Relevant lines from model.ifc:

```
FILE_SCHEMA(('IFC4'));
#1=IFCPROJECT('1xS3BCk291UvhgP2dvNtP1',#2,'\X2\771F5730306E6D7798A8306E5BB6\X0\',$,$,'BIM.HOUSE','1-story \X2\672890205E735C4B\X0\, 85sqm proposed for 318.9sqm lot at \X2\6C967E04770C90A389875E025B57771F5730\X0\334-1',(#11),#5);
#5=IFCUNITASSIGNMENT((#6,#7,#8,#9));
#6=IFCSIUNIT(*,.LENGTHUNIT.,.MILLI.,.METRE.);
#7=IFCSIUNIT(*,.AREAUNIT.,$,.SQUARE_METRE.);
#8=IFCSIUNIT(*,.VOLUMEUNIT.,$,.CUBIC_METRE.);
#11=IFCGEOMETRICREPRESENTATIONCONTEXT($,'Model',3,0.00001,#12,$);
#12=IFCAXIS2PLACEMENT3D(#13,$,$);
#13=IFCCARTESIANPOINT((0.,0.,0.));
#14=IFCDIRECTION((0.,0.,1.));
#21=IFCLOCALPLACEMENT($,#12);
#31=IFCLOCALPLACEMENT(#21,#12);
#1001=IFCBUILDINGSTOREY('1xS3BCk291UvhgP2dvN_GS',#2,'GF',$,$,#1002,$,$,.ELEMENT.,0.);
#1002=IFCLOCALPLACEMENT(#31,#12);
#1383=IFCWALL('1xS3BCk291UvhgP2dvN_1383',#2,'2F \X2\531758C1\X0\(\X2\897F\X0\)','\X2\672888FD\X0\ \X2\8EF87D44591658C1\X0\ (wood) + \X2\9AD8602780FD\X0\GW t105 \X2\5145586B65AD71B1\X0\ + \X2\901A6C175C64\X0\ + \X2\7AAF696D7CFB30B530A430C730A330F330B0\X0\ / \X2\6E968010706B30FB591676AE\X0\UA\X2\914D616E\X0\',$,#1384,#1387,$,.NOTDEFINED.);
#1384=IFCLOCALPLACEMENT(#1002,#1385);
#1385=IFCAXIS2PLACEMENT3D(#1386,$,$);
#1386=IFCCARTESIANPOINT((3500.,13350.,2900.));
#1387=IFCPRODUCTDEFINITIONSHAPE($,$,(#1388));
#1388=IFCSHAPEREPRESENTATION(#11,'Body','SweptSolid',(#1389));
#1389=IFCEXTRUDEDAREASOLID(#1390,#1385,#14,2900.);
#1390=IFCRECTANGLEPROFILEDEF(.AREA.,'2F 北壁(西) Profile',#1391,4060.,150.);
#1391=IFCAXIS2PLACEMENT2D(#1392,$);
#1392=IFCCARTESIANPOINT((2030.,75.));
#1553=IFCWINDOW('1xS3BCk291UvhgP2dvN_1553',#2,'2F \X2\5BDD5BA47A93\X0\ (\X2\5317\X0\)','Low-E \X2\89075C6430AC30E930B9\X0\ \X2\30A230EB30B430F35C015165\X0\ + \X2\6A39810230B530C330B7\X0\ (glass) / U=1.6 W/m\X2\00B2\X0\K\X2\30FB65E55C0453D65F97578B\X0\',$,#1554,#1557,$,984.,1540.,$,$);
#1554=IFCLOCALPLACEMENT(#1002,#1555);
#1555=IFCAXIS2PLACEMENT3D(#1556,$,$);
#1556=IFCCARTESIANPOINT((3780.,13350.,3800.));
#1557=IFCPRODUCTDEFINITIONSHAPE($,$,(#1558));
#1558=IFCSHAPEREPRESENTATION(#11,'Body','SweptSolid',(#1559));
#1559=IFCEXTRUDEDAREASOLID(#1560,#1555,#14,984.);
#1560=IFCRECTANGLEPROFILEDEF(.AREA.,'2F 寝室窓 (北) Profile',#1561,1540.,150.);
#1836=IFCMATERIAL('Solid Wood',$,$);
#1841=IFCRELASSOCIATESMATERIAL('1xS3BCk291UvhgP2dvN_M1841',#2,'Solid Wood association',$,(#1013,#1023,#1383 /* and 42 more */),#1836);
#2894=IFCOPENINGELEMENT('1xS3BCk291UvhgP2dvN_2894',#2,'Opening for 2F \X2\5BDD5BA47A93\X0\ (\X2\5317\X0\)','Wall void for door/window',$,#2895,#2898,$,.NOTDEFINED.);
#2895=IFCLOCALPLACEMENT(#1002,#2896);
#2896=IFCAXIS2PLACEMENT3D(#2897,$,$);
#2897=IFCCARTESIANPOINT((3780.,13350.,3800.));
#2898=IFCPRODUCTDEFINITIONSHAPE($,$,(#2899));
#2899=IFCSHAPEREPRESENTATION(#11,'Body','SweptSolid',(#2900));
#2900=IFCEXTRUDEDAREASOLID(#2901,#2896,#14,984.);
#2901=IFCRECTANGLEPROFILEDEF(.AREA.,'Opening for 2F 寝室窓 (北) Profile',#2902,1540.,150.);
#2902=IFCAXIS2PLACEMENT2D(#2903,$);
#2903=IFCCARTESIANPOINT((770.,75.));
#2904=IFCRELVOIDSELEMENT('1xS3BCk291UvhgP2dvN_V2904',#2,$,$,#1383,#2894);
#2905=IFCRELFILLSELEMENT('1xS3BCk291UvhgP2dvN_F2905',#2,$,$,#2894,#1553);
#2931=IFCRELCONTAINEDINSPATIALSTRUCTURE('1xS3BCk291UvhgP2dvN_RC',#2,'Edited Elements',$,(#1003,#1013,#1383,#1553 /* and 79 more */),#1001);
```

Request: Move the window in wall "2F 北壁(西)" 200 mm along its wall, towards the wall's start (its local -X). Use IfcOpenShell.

```python
import ifcopenshell
import ifcopenshell.api.geometry
import ifcopenshell.util.placement

model = ifcopenshell.open("model.ifc")

window = model.by_guid("1xS3BCk291UvhgP2dvN_1553")
opening = window.FillsVoids[0].RelatingOpeningElement
wall = opening.VoidsElements[0].RelatingBuildingElement

wall_matrix = ifcopenshell.util.placement.get_local_placement(wall.ObjectPlacement)
shift = wall_matrix[:3, 0] * -200.0
before = ifcopenshell.util.placement.get_local_placement(window.ObjectPlacement)[:3, 3].copy()

# The window is not placed relative to its opening, so move both.
for product in (opening, window):
    matrix = ifcopenshell.util.placement.get_local_placement(product.ObjectPlacement)
    matrix[:3, 3] += shift
    ifcopenshell.api.geometry.edit_object_placement(model, product=product, matrix=matrix, is_si=False)

after = ifcopenshell.util.placement.get_local_placement(window.ObjectPlacement)[:3, 3]
print("window moved by", (after - before).round(3) + 0.0)

model.write("model_edited.ifc")
```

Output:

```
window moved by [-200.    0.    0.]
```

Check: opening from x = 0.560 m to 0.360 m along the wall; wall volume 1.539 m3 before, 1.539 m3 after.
